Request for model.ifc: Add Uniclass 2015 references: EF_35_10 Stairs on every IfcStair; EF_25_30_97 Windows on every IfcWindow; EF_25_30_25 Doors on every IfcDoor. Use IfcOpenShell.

First a look at what the model holds.

```python
import ifcopenshell

model = ifcopenshell.open("model.ifc")
print(model.schema)
print("classifications:", [c.Name for c in model.by_type("IfcClassification")])
for ifc_class in ("IfcDoor", "IfcRoof", "IfcStair", "IfcWall", "IfcWindow"):
    print(ifc_class, len(model.by_type(ifc_class)))
```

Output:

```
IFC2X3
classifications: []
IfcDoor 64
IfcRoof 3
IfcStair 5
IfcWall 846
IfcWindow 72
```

```python
import ifcopenshell
import ifcopenshell.api.classification

model = ifcopenshell.open("model.ifc")

# IFC2X3 requires Source and Edition and has no link from the project to the system.
system = model.create_entity("IfcClassification", Source="NBS", Edition="2015", Name="Uniclass 2015")

codes = {
    "IfcStair": ("EF_35_10", "Stairs"),
    "IfcWindow": ("EF_25_30_97", "Windows"),
    "IfcDoor": ("EF_25_30_25", "Doors"),
}
for ifc_class, (code, name) in codes.items():
    products = model.by_type(ifc_class)
    ifcopenshell.api.classification.add_reference(
        model, products=products, classification=system, identification=code, name=name
    )
    print(code, len(products))

model.write("model_updated.ifc")
```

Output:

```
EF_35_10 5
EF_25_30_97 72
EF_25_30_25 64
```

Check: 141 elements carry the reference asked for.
